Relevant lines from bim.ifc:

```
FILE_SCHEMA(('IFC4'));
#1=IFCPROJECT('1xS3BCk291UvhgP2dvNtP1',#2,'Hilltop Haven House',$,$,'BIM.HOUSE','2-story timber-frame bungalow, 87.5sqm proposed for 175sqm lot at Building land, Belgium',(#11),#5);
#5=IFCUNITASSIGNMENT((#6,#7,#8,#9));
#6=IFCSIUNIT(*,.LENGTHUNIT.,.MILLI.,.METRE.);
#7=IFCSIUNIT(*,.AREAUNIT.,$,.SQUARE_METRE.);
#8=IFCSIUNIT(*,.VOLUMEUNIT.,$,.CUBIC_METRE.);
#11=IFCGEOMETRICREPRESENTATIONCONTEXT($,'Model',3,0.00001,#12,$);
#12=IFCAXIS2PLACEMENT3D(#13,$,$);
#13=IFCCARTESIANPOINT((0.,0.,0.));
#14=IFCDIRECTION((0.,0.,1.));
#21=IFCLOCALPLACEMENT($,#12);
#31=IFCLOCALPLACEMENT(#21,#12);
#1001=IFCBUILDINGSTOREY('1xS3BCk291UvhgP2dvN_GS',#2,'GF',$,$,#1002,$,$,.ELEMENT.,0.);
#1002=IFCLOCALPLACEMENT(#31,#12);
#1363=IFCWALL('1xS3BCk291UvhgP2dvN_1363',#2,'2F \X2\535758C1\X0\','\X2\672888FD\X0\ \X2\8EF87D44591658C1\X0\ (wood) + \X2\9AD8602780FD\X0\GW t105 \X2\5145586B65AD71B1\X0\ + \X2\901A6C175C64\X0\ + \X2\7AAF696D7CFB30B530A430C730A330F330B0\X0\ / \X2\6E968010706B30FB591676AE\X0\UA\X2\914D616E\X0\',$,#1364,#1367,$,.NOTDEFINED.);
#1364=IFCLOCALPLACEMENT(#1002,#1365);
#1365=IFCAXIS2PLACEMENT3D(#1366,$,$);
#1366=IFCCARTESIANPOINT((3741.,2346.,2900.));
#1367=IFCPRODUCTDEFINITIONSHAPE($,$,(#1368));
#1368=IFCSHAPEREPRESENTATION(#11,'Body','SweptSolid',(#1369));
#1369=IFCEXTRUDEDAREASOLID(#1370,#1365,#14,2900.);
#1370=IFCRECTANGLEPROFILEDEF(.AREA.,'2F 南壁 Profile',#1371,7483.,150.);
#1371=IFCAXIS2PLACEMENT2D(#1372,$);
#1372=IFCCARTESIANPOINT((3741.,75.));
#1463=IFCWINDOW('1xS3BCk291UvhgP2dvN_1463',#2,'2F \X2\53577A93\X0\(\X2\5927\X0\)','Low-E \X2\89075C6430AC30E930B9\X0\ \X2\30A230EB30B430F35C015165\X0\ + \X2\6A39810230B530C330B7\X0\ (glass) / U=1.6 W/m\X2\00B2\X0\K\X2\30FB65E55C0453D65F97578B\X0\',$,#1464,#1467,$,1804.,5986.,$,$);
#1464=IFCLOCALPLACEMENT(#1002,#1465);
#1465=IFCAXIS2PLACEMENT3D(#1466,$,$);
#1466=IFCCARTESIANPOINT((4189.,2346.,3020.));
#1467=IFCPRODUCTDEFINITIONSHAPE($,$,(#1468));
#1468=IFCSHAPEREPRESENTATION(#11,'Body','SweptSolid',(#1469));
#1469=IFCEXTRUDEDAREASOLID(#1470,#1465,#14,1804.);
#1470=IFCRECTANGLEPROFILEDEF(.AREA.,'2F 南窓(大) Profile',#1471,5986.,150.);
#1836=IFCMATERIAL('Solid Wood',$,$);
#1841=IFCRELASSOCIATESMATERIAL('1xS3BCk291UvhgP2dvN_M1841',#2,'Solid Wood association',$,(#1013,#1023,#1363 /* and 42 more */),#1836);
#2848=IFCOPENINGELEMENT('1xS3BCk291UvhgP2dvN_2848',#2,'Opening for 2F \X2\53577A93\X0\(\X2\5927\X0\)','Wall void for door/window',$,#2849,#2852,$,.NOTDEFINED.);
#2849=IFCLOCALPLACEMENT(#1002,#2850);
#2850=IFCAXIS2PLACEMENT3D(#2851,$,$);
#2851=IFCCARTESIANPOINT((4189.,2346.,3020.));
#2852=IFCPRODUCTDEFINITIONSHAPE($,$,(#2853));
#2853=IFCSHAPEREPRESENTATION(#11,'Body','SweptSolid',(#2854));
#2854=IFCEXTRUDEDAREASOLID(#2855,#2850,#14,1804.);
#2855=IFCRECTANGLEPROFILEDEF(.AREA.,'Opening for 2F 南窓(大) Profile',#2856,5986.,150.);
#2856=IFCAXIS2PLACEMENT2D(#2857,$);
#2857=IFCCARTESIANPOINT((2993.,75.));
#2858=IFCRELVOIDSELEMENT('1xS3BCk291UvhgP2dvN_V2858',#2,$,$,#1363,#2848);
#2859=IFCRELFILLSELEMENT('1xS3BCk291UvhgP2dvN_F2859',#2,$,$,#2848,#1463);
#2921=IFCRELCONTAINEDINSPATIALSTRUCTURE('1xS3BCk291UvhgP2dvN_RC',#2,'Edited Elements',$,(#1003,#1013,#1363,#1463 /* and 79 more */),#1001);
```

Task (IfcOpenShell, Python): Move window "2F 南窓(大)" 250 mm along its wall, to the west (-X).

```python
import ifcopenshell
import ifcopenshell.api.geometry
import ifcopenshell.util.placement

model = ifcopenshell.open("bim.ifc")

window = model.by_id(1463)
opening = window.FillsVoids[0].RelatingOpeningElement
wall = opening.VoidsElements[0].RelatingBuildingElement

wall_matrix = ifcopenshell.util.placement.get_local_placement(wall.ObjectPlacement)
shift = wall_matrix[:3, 0] * -250.0
before = ifcopenshell.util.placement.get_local_placement(window.ObjectPlacement)[:3, 3].copy()

# The window is not placed relative to its opening, so move both.
for product in (opening, window):
    matrix = ifcopenshell.util.placement.get_local_placement(product.ObjectPlacement)
    matrix[:3, 3] += shift
    ifcopenshell.api.geometry.edit_object_placement(model, product=product, matrix=matrix, is_si=False)

after = ifcopenshell.util.placement.get_local_placement(window.ObjectPlacement)[:3, 3]
print("window moved by", (after - before).round(3) + 0.0)

model.write("bim_rev.ifc")
```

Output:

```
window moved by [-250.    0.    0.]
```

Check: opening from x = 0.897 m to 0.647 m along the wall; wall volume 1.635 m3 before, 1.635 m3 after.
